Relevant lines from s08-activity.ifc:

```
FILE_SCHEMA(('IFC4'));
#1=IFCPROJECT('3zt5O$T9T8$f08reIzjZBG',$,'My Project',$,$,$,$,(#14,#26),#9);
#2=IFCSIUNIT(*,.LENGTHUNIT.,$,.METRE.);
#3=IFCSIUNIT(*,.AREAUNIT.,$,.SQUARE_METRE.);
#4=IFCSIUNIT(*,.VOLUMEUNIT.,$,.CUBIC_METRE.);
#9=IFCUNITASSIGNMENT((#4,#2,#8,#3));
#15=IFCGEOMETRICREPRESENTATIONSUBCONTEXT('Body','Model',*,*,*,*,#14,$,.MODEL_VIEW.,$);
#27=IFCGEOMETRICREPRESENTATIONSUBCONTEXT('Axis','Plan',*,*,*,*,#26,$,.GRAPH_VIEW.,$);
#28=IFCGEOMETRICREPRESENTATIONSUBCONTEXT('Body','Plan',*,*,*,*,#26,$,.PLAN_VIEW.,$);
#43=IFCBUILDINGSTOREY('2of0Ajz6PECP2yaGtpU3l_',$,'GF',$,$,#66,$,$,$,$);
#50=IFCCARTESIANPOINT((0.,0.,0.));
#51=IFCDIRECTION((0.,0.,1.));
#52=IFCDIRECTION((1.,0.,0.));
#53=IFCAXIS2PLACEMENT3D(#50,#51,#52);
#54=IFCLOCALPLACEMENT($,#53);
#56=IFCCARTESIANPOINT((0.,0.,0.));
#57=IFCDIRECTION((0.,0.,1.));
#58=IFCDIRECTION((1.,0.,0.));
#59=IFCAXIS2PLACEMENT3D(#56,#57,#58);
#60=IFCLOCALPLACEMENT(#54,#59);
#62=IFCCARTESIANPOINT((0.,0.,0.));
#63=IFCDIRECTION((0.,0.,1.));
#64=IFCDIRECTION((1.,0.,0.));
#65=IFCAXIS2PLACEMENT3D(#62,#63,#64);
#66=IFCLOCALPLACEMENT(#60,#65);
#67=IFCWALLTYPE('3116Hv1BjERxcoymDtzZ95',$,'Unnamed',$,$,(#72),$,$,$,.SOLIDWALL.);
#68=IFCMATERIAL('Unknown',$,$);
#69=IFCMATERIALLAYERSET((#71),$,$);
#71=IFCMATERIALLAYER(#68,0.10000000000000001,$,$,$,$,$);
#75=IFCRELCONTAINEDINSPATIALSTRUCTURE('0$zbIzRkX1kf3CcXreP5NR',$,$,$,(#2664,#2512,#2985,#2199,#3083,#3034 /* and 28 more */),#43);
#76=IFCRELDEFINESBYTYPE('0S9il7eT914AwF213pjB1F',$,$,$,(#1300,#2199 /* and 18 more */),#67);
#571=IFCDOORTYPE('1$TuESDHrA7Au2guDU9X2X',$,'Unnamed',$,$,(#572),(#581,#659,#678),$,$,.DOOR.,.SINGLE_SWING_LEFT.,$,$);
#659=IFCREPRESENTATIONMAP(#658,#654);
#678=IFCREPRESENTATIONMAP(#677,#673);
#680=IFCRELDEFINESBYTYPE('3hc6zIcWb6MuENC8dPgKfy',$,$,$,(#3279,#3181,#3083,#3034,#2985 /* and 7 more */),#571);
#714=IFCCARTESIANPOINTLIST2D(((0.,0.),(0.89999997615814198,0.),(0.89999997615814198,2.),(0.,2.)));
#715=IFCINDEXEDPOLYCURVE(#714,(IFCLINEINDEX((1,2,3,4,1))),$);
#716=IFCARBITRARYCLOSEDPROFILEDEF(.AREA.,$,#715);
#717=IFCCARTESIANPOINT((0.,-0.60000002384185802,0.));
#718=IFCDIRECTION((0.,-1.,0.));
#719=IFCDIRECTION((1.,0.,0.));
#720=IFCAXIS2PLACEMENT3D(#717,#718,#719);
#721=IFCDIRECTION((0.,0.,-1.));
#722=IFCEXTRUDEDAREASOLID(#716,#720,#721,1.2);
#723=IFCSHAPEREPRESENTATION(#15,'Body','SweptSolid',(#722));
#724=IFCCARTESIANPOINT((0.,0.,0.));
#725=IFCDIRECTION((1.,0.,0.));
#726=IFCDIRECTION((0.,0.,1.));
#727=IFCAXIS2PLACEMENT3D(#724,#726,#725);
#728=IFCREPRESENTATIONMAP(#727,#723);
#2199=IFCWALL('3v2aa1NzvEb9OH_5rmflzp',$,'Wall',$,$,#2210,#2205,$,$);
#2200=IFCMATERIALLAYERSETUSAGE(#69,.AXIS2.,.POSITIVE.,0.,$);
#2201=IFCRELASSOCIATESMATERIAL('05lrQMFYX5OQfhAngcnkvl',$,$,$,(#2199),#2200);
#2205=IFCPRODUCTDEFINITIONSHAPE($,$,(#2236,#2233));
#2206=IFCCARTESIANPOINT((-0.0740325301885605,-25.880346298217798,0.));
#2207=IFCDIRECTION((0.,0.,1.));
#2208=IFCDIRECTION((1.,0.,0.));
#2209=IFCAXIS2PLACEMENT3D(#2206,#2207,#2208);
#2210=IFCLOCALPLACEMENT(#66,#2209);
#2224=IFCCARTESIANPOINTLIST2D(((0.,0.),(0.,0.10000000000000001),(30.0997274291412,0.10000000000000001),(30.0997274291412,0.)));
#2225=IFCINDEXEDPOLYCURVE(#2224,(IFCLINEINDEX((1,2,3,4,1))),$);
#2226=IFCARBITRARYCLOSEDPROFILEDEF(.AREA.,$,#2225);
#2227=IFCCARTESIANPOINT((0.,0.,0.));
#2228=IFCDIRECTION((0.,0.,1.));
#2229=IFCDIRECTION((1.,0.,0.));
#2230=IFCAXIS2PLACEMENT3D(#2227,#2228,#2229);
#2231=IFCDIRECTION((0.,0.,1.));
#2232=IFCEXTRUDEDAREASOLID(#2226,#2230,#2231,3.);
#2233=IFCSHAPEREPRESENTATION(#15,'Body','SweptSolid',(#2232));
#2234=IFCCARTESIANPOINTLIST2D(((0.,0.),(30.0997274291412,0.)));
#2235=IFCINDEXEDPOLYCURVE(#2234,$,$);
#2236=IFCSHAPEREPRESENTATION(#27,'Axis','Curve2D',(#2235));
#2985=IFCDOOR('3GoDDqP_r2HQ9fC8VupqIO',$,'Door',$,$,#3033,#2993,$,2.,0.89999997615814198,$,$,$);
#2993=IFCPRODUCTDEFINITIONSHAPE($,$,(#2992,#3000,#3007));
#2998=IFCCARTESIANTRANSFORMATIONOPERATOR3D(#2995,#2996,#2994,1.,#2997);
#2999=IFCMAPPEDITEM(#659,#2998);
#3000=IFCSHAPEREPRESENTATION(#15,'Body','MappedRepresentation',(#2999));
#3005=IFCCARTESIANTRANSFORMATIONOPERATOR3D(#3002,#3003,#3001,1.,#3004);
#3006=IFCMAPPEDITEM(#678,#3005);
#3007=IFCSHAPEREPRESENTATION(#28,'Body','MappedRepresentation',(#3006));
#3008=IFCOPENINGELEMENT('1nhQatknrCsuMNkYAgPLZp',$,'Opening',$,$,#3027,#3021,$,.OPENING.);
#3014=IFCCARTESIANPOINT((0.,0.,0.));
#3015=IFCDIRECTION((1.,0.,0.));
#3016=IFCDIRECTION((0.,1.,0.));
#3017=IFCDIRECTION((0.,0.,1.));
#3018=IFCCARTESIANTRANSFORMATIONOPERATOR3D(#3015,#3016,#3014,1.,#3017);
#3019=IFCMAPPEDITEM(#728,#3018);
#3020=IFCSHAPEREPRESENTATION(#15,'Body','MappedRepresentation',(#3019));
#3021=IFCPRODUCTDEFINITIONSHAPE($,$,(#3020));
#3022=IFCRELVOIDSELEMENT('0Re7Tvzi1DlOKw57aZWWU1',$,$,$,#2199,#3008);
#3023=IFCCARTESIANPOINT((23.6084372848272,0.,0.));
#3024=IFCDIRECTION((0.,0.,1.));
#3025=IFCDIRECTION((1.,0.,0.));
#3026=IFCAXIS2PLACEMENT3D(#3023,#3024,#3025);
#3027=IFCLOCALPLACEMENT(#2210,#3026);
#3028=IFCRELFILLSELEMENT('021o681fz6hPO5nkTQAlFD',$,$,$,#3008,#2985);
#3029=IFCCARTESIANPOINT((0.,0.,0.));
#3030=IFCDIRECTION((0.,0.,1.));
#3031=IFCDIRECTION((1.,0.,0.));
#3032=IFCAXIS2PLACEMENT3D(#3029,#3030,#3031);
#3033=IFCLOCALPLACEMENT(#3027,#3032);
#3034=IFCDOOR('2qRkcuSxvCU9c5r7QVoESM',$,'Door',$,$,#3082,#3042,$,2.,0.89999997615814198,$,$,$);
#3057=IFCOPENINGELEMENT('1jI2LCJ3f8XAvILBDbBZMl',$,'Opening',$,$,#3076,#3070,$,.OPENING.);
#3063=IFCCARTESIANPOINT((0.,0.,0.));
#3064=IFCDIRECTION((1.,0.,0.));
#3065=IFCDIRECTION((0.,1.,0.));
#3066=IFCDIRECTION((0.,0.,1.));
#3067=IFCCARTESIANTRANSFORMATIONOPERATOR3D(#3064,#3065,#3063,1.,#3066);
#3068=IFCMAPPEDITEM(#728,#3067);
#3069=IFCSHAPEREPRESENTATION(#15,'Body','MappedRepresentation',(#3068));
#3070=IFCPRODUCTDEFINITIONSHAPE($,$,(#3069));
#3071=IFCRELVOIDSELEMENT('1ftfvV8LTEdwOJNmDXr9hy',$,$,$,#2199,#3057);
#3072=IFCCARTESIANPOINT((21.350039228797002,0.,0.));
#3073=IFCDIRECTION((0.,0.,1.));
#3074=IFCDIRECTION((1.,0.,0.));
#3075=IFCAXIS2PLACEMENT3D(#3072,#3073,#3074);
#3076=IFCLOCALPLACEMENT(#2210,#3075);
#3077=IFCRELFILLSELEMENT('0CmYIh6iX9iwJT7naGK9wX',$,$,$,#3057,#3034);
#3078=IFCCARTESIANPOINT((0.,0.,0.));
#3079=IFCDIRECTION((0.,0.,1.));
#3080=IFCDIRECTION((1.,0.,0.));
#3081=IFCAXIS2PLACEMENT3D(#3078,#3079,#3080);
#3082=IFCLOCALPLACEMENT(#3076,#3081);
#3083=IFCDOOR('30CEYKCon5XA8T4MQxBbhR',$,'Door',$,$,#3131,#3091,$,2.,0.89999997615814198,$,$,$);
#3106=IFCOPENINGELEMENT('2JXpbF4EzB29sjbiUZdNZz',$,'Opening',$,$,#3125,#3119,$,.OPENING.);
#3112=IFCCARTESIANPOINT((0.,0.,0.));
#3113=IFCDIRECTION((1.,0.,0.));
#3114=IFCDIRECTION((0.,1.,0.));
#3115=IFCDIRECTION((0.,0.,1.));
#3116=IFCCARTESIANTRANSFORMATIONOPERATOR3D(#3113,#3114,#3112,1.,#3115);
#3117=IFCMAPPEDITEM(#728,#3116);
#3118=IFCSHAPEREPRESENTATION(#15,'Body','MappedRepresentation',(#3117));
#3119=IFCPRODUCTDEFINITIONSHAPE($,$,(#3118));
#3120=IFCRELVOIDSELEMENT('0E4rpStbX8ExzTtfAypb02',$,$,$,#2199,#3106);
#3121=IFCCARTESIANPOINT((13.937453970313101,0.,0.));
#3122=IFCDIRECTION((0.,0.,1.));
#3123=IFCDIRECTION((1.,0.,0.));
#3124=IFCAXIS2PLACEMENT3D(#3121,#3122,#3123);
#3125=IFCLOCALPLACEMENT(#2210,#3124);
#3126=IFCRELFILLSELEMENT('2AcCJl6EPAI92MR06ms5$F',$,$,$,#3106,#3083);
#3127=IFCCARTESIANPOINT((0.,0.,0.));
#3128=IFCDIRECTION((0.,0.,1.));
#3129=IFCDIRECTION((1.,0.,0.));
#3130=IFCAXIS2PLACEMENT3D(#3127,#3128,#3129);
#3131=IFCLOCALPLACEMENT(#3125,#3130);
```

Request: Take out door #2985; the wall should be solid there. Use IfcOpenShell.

```python
import ifcopenshell
import ifcopenshell.api.feature
import ifcopenshell.api.root
import ifcopenshell.geom
import ifcopenshell.util.shape

model = ifcopenshell.open("s08-activity.ifc")
settings = ifcopenshell.geom.settings()


def volume(element):
    """Net volume in cubic metres, openings subtracted."""
    shape = ifcopenshell.geom.create_shape(settings, element)
    return ifcopenshell.util.shape.get_volume(shape.geometry)


door = model.by_guid("3GoDDqP_r2HQ9fC8VupqIO")
opening = door.FillsVoids[0].RelatingOpeningElement
wall = opening.VoidsElements[0].RelatingBuildingElement
before = volume(wall)

ifcopenshell.api.root.remove_product(model, product=door)
ifcopenshell.api.feature.remove_feature(model, feature=opening)

after = volume(wall)

print(f"wall volume {before:.3f} -> {after:.3f} m3")

model.write("s08-activity_edited.ifc")
```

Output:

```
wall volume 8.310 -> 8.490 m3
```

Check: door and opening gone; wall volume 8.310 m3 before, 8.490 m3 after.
